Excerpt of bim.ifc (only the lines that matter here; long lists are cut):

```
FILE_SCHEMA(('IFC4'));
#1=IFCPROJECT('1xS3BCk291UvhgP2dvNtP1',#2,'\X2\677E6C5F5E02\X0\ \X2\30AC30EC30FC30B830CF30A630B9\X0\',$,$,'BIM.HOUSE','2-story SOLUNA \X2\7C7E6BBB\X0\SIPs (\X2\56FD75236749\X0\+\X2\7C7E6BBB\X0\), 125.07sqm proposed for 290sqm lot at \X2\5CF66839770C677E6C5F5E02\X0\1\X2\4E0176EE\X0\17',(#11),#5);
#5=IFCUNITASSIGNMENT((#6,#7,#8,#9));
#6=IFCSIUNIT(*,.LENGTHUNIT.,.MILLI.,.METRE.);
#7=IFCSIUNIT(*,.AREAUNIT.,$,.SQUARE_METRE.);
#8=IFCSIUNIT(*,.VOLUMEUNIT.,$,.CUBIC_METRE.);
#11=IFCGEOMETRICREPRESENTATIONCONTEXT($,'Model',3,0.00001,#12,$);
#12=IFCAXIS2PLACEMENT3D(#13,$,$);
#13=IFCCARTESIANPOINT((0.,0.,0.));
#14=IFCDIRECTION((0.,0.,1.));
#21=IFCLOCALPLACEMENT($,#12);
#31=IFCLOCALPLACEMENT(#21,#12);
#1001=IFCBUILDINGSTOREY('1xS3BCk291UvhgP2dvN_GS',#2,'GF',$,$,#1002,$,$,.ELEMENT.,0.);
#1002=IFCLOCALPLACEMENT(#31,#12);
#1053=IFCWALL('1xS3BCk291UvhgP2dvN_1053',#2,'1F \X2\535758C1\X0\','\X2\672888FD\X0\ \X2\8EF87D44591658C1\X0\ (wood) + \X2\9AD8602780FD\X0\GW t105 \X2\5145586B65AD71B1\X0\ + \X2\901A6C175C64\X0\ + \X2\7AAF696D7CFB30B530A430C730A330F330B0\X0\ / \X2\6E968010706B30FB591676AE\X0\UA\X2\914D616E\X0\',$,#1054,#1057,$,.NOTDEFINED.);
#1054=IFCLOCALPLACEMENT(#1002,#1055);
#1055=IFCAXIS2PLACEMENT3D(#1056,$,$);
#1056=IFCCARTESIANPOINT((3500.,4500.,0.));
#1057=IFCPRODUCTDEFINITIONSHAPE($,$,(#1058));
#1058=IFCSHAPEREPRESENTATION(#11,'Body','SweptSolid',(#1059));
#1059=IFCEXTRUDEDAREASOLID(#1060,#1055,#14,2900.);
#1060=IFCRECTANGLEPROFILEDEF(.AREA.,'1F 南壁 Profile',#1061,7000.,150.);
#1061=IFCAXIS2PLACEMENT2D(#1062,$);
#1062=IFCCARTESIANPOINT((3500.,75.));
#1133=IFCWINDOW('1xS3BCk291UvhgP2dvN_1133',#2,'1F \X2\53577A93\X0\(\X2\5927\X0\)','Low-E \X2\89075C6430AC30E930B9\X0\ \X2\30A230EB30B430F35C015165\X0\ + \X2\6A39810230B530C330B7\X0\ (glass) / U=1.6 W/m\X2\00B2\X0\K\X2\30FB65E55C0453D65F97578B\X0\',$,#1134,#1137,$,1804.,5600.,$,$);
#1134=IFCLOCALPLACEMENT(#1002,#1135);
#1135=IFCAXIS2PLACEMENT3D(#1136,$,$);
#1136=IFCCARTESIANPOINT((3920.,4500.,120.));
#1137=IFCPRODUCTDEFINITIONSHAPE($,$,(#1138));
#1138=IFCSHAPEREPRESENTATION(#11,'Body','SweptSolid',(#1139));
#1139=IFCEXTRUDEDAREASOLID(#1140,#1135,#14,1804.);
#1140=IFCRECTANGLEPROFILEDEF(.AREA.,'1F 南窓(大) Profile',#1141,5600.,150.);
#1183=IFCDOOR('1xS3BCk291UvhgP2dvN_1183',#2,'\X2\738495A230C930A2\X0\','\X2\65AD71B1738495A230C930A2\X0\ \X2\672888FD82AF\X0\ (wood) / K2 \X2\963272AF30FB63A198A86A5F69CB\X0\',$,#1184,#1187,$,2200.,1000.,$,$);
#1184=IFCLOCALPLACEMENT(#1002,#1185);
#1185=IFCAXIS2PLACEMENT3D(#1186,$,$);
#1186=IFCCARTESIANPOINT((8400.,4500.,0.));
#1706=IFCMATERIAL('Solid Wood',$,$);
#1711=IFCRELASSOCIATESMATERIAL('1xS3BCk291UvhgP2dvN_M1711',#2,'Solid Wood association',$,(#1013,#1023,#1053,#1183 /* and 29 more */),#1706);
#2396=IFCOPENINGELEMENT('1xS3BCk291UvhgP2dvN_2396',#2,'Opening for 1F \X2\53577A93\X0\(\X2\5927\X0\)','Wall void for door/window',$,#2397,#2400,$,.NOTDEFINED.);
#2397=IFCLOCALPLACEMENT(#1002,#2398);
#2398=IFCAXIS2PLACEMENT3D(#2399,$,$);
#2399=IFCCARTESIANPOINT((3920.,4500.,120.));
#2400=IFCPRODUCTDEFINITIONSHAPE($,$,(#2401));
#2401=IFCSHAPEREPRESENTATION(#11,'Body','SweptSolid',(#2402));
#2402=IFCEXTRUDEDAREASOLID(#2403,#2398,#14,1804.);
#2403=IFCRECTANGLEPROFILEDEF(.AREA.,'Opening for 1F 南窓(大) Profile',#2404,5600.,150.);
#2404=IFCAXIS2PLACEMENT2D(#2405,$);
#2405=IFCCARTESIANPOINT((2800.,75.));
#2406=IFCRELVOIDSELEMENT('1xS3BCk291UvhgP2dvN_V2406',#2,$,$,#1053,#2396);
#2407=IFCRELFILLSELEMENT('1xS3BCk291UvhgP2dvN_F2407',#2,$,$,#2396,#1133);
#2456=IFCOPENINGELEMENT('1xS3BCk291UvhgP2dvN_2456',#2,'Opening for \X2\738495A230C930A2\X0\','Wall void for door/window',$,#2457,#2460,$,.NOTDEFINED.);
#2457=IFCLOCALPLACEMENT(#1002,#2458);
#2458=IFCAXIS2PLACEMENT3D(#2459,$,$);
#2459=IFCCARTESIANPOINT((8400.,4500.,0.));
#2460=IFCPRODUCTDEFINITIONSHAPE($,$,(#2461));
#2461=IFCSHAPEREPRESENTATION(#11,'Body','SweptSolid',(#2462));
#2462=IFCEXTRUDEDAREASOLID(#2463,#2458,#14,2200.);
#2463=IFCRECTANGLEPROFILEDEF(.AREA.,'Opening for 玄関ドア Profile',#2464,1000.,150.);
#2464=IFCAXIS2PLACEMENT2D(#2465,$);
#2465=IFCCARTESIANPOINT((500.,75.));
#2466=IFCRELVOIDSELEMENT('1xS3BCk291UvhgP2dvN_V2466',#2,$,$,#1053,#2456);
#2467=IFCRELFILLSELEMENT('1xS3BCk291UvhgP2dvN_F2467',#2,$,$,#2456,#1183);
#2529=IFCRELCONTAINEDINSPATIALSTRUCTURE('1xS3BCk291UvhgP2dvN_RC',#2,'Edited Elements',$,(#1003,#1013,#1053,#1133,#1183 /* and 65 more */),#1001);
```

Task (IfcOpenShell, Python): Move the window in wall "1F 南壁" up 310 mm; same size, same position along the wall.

```python
import numpy as np
import ifcopenshell
import ifcopenshell.api.geometry
import ifcopenshell.util.placement
import ifcopenshell.util.unit

model = ifcopenshell.open("bim.ifc")
unit_scale = ifcopenshell.util.unit.calculate_unit_scale(model)

window = model.by_id(1133)
opening = window.FillsVoids[0].RelatingOpeningElement
dz = 310.0

shift = np.array([0.0, 0.0, dz])
# The window is not placed relative to its opening, so move both.
for product in (opening, window):
    matrix = ifcopenshell.util.placement.get_local_placement(product.ObjectPlacement)
    matrix[:3, 3] += shift
    ifcopenshell.api.geometry.edit_object_placement(model, product=product, matrix=matrix, is_si=False)

print(f"moved by {dz * unit_scale:+.3f} m")

model.write("bim_edited.ifc")
```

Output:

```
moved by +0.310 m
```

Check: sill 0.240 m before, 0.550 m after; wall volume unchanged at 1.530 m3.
